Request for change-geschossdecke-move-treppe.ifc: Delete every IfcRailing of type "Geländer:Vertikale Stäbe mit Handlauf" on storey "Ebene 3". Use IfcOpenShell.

First a look at what the model holds.

```python
import ifcopenshell
import ifcopenshell.util.element

model = ifcopenshell.open("change-geschossdecke-move-treppe.ifc")
print(model.schema)
storey = next(s for s in model.by_type("IfcBuildingStorey") if s.Name == "Ebene 3")
railings = [e for e in ifcopenshell.util.element.get_decomposition(storey) if e.is_a("IfcRailing")]
seen = {}
for e in railings:
    element_type = ifcopenshell.util.element.get_type(e)
    name = element_type.Name if element_type not in (None, e) else None
    seen[name] = seen.get(name, 0) + 1
for name, count in sorted(seen.items(), key=str):
    print(count, "x", name)
```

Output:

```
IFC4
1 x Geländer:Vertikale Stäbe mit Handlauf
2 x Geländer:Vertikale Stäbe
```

```python
import ifcopenshell
import ifcopenshell.api.root
import ifcopenshell.util.element

model = ifcopenshell.open("change-geschossdecke-move-treppe.ifc")

storey = next(s for s in model.by_type("IfcBuildingStorey") if s.Name == "Ebene 3")
railings = [e for e in ifcopenshell.util.element.get_decomposition(storey) if e.is_a("IfcRailing")]
targets = [e for e in railings if (t := ifcopenshell.util.element.get_type(e)) not in (None, e) and t.Name == "Geländer:Vertikale Stäbe mit Handlauf"]

for e in targets:
    ifcopenshell.api.root.remove_product(model, product=e)
print(len(targets), "removed")

model.write("change-geschossdecke-move-treppe_edited.ifc")
```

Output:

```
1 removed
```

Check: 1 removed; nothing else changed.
